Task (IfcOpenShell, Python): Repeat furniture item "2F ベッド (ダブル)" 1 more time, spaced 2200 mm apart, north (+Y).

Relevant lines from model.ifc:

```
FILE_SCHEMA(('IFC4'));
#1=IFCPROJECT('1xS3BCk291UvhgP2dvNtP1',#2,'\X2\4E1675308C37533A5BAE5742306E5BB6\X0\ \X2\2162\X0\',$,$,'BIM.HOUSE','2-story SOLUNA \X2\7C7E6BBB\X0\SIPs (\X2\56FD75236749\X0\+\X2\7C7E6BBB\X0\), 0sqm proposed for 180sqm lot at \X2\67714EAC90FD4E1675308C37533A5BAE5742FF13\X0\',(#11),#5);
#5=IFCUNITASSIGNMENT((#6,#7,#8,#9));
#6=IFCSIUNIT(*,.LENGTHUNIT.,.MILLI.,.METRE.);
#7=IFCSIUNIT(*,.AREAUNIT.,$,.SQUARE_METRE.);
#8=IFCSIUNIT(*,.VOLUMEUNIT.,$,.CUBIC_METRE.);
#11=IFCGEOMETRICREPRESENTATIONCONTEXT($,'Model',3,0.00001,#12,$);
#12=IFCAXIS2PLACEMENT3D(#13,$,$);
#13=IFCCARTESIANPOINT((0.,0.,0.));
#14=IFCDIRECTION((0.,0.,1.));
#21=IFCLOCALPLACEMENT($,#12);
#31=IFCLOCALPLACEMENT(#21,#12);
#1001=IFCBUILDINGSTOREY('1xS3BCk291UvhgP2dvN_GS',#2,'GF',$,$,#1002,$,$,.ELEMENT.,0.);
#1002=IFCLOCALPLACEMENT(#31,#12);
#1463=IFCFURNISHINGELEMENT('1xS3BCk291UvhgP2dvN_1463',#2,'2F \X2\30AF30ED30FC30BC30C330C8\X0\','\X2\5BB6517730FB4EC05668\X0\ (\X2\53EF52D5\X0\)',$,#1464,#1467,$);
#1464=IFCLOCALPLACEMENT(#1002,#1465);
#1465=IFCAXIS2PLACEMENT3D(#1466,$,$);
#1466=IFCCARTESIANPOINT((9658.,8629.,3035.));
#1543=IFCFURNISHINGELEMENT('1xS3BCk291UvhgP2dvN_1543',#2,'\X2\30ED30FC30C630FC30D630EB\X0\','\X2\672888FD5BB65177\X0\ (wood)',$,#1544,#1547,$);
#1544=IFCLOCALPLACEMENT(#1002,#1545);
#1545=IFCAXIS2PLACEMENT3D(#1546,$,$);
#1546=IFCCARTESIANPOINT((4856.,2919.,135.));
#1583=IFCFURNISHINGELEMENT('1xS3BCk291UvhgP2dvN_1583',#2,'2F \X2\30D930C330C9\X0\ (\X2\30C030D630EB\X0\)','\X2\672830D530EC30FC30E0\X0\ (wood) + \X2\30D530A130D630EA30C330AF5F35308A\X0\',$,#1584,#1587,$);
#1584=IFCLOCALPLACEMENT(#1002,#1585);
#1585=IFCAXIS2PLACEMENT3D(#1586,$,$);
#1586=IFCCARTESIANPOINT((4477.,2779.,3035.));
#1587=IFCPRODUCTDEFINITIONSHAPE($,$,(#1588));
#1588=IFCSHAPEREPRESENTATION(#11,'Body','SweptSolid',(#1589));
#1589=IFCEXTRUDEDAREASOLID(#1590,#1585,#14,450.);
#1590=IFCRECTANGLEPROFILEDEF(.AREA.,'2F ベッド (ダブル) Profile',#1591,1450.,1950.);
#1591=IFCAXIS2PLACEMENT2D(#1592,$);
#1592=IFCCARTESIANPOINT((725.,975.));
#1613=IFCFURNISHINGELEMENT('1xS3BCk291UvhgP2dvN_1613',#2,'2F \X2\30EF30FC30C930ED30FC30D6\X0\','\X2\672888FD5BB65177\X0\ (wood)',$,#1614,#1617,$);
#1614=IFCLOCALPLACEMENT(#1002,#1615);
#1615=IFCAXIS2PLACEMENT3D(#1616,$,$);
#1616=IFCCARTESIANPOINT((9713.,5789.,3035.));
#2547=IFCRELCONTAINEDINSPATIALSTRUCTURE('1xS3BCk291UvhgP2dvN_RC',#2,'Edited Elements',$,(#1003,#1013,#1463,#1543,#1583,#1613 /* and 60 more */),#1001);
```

```python
import numpy as np
import ifcopenshell
import ifcopenshell.api.geometry
import ifcopenshell.api.root
import ifcopenshell.util.element
import ifcopenshell.util.placement

model = ifcopenshell.open("model.ifc")


def reuse_history(source, copy):
    """copy_class also copies each property set's owner history, people and application; keep the originals."""
    for rel in copy.IsDefinedBy:
        if rel.is_a("IfcRelDefinesByProperties") and (history := rel.RelatingPropertyDefinition.OwnerHistory):
            rel.RelatingPropertyDefinition.OwnerHistory = source.OwnerHistory
            ifcopenshell.util.element.remove_deep2(model, history)


source = model.by_guid("1xS3BCk291UvhgP2dvN_1583")
base = ifcopenshell.util.placement.get_local_placement(source.ObjectPlacement)
step = np.array([0.0, 1.0, 0.0]) * 2200.0

for i in range(1, 2):
    copy = ifcopenshell.api.root.copy_class(model, product=source)
    copy.Representation = ifcopenshell.util.element.copy_deep(
        model, source.Representation, exclude=["IfcGeometricRepresentationContext", "IfcRepresentationMap"]
    )
    reuse_history(source, copy)
    matrix = base.copy()
    matrix[:3, 3] += i * step
    print("added at", matrix[:3, 3].round(3) + 0.0)
    ifcopenshell.api.geometry.edit_object_placement(model, product=copy, matrix=matrix, is_si=False)

model.write("model_v2.ifc")
```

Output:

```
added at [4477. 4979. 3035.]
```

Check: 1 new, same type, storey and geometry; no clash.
